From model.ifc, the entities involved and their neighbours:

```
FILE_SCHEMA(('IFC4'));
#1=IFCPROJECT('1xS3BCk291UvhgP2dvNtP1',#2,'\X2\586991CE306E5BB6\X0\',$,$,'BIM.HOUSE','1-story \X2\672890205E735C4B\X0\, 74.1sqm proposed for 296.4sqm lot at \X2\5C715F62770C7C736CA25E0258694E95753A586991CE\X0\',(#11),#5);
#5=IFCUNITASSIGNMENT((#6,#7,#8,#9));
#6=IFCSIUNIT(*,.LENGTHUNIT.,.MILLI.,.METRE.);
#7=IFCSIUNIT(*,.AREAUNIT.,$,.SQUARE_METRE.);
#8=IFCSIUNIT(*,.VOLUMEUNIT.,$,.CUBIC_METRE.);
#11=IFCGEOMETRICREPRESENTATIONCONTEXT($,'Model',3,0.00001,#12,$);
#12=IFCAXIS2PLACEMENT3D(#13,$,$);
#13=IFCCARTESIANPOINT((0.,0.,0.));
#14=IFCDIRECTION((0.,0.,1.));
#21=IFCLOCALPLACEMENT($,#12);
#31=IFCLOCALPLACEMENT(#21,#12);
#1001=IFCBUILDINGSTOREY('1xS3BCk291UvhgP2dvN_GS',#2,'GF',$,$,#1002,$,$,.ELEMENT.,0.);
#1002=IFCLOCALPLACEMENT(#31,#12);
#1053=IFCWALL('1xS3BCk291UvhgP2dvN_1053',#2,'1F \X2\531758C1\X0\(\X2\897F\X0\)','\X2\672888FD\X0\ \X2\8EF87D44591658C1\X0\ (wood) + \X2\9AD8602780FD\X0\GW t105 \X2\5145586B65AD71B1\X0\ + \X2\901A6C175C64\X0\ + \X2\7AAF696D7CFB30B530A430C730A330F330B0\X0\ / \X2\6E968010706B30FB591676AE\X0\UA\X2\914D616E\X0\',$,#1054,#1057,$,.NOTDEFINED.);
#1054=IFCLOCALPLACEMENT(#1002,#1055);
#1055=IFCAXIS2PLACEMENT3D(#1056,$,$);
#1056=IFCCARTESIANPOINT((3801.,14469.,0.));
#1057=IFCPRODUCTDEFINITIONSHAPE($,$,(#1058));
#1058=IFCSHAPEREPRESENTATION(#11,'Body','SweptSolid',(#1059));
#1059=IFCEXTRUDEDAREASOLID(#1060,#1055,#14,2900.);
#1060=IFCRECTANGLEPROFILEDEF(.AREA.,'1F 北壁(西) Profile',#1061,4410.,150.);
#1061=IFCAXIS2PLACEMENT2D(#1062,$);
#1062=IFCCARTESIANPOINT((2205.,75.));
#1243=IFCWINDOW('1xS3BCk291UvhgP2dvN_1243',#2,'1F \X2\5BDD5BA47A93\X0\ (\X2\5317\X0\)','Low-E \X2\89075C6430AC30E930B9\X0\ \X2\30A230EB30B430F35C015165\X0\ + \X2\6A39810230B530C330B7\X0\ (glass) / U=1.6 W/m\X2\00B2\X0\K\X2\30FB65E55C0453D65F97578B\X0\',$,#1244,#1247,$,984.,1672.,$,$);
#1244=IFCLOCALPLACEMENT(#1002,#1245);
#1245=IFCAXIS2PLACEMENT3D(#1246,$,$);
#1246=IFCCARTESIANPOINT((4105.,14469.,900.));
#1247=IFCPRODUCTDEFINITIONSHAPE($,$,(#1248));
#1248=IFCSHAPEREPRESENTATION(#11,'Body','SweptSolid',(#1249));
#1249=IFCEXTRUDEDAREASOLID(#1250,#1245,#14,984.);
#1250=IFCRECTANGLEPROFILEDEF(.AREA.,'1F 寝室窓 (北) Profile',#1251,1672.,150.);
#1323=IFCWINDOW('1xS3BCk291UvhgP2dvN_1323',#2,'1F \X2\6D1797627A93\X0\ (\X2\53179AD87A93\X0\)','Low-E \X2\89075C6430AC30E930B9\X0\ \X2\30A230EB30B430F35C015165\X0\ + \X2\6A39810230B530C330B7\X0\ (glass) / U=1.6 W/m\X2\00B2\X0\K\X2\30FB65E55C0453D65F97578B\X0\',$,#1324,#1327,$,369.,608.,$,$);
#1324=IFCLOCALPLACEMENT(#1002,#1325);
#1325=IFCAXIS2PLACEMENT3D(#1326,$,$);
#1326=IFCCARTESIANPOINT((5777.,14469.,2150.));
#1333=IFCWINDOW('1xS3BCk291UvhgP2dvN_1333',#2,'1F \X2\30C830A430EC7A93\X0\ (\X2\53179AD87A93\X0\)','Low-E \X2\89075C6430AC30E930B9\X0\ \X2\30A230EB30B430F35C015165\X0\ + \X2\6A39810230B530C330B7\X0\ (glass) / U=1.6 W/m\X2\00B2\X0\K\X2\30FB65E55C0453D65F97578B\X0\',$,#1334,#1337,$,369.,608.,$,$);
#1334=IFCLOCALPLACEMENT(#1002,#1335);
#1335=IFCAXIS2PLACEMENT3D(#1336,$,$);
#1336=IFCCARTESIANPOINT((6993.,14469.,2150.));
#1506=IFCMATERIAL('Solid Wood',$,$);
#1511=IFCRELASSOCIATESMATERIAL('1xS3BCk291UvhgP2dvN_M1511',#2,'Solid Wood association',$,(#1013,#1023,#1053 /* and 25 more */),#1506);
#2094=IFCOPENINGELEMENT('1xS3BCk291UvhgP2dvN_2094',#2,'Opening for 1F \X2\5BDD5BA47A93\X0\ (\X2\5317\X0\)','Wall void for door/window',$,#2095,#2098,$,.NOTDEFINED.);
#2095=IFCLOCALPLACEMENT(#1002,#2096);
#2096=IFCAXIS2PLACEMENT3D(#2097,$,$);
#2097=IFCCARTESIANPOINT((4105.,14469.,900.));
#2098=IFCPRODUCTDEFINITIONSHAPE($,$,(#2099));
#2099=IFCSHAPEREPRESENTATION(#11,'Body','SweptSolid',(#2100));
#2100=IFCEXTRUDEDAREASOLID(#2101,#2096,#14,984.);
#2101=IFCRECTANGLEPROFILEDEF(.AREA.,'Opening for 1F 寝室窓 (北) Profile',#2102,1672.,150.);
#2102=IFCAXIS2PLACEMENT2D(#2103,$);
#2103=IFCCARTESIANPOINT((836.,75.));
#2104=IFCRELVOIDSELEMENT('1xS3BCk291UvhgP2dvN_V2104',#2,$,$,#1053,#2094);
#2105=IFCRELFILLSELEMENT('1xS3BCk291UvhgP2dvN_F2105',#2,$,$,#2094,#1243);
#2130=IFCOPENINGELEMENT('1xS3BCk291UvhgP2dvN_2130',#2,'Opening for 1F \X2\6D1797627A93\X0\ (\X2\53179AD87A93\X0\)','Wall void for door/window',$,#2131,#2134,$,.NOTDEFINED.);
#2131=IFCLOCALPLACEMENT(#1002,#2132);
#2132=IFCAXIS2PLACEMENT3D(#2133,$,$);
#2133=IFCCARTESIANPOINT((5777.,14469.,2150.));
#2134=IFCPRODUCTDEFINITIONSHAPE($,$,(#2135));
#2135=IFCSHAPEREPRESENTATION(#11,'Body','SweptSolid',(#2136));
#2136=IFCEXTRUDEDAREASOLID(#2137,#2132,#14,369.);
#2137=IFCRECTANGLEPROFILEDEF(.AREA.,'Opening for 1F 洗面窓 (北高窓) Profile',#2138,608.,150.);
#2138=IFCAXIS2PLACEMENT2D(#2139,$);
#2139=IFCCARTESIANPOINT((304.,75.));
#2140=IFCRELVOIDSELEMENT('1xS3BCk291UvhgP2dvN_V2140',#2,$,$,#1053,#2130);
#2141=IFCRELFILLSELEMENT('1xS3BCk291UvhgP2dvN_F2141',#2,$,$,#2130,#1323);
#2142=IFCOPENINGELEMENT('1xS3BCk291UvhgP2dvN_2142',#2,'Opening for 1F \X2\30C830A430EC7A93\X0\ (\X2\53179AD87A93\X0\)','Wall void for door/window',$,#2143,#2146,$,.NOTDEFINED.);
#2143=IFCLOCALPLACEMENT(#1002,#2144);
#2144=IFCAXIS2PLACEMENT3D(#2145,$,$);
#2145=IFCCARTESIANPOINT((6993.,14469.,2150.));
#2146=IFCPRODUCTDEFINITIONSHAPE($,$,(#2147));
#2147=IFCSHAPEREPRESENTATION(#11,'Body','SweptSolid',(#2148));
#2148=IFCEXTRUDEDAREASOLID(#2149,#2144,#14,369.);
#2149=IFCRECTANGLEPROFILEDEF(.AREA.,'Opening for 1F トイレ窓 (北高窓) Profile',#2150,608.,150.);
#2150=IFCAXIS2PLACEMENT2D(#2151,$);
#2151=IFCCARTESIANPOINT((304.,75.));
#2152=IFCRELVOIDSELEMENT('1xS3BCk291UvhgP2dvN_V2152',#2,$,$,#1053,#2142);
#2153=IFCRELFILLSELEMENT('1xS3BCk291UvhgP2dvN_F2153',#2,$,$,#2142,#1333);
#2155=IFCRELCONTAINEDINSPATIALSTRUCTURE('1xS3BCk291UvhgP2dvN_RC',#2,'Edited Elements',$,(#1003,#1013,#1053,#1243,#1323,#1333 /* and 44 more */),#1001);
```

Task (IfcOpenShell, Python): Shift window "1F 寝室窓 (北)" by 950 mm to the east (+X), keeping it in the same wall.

```python
import ifcopenshell
import ifcopenshell.api.geometry
import ifcopenshell.util.placement

model = ifcopenshell.open("model.ifc")

window = model.by_guid("1xS3BCk291UvhgP2dvN_1243")
opening = window.FillsVoids[0].RelatingOpeningElement
wall = opening.VoidsElements[0].RelatingBuildingElement

wall_matrix = ifcopenshell.util.placement.get_local_placement(wall.ObjectPlacement)
shift = wall_matrix[:3, 0] * 950.0
before = ifcopenshell.util.placement.get_local_placement(window.ObjectPlacement)[:3, 3].copy()

# The window is not placed relative to its opening, so move both.
for product in (opening, window):
    matrix = ifcopenshell.util.placement.get_local_placement(product.ObjectPlacement)
    matrix[:3, 3] += shift
    ifcopenshell.api.geometry.edit_object_placement(model, product=product, matrix=matrix, is_si=False)

after = ifcopenshell.util.placement.get_local_placement(window.ObjectPlacement)[:3, 3]
print("window moved by", (after - before).round(3) + 0.0)

model.write("model_rev.ifc")
```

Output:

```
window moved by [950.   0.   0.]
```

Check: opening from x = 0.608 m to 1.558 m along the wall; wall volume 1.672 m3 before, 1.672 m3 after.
